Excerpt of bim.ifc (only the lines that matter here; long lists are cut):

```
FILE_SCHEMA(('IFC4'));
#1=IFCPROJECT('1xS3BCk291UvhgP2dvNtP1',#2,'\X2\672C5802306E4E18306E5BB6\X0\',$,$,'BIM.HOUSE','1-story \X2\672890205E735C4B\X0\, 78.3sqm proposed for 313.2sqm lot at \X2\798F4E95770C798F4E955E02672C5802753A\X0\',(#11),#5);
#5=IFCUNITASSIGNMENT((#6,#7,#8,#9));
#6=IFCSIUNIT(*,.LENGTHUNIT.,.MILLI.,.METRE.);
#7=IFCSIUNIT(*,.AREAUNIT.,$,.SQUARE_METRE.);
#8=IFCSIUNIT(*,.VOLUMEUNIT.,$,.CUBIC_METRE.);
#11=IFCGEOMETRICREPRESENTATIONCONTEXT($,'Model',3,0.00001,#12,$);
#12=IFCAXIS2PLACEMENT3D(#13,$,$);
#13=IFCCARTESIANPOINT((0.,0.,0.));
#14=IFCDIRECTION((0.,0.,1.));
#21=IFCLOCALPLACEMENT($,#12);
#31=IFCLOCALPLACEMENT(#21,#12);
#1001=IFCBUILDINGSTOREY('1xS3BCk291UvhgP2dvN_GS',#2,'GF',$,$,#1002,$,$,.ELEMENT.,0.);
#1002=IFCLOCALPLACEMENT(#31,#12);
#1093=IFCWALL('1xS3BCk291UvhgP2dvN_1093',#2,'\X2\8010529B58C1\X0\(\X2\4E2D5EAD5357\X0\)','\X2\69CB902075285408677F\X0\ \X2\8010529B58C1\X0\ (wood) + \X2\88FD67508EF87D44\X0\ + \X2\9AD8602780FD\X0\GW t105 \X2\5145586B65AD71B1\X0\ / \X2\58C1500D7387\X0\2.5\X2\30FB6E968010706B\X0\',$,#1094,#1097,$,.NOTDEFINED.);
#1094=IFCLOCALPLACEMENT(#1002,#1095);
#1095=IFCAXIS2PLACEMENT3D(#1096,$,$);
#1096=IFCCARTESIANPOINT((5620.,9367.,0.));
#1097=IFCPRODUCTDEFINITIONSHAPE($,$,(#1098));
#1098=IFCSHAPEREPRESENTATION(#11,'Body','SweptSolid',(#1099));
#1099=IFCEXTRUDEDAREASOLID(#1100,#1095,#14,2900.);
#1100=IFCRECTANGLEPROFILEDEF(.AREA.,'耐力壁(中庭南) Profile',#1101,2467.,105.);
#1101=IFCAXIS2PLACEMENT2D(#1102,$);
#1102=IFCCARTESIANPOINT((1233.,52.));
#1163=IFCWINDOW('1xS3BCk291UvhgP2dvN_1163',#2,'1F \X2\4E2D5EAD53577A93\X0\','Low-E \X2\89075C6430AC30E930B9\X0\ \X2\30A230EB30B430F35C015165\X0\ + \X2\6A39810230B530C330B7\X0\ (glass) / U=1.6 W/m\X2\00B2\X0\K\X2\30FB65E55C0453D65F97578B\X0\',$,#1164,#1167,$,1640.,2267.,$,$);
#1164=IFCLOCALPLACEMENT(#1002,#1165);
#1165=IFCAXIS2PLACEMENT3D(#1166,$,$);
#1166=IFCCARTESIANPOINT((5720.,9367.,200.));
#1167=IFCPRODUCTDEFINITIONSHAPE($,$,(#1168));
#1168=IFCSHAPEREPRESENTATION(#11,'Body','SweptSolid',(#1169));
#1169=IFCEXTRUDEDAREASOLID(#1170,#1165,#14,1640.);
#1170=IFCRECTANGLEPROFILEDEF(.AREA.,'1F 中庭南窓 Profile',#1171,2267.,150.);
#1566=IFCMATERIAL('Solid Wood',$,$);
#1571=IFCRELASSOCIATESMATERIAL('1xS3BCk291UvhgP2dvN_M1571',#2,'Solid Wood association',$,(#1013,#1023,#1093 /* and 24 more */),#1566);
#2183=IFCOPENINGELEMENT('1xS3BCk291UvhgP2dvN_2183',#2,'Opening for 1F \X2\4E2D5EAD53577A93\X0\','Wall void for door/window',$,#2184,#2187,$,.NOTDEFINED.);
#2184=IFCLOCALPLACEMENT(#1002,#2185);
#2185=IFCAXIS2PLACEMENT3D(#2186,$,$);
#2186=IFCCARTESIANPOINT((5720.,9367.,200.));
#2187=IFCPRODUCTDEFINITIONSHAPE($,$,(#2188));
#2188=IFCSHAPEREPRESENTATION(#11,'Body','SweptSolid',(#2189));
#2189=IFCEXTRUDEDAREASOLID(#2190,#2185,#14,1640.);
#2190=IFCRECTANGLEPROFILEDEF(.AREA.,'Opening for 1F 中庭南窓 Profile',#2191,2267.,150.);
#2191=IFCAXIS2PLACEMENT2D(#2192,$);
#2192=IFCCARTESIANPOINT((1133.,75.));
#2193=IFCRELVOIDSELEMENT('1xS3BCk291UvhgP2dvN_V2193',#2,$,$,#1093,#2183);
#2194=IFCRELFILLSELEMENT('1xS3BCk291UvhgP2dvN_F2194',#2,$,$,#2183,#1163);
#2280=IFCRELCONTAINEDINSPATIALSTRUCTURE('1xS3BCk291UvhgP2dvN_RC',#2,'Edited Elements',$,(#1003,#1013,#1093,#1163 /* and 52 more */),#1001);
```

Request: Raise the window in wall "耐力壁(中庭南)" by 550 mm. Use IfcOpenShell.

```python
import numpy as np
import ifcopenshell
import ifcopenshell.api.geometry
import ifcopenshell.util.placement
import ifcopenshell.util.unit

model = ifcopenshell.open("bim.ifc")
unit_scale = ifcopenshell.util.unit.calculate_unit_scale(model)

window = model.by_guid("1xS3BCk291UvhgP2dvN_1163")
opening = window.FillsVoids[0].RelatingOpeningElement
dz = 550.0

shift = np.array([0.0, 0.0, dz])
# The window is not placed relative to its opening, so move both.
for product in (opening, window):
    matrix = ifcopenshell.util.placement.get_local_placement(product.ObjectPlacement)
    matrix[:3, 3] += shift
    ifcopenshell.api.geometry.edit_object_placement(model, product=product, matrix=matrix, is_si=False)

print(f"moved by {dz * unit_scale:+.3f} m")

model.write("bim_edited.ifc")
```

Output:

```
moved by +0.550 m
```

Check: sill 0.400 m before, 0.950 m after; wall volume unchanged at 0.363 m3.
